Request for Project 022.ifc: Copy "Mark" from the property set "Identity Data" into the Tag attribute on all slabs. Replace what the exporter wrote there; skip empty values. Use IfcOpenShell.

First a look at what the model holds.

```python
import ifcopenshell
import ifcopenshell.util.element

model = ifcopenshell.open("Project 022.ifc")
print(model.schema)
slabs = model.by_type("IfcSlab")
print(len(slabs), "slabs")
for e in slabs[:8]:
    source = ifcopenshell.util.element.get_pset(e, "Identity Data", "Mark")
    target = e.Tag
    print(e.id(), repr(source), repr(target), sep=" | ")
```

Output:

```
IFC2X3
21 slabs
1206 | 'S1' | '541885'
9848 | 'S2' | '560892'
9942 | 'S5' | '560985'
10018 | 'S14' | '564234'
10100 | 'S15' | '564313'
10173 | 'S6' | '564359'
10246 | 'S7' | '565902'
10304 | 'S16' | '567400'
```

```python
import ifcopenshell
import ifcopenshell.util.element

model = ifcopenshell.open("Project 022.ifc")

count = 0
for e in model.by_type("IfcSlab"):
    value = ifcopenshell.util.element.get_pset(e, "Identity Data", "Mark")
    current = e.Tag
    if not value or not value.strip() or current == value:
        continue
    e.Tag = value
    count += 1

print(count, "slabs updated")

model.write("Project 022_updated.ifc")
```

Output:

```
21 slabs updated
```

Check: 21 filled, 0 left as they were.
